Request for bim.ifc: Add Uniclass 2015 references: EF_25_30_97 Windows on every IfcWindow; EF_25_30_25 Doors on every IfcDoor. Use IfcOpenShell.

First a look at what the model holds.

```python
import ifcopenshell

model = ifcopenshell.open("bim.ifc")
print(model.schema)
print("classifications:", [c.Name for c in model.by_type("IfcClassification")])
for ifc_class in ("IfcDoor", "IfcRoof", "IfcStair", "IfcWall", "IfcWindow"):
    print(ifc_class, len(model.by_type(ifc_class)))
```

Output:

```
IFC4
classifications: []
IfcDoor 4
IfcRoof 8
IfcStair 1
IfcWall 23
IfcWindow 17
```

```python
import ifcopenshell
import ifcopenshell.api.classification

model = ifcopenshell.open("bim.ifc")

system = ifcopenshell.api.classification.add_classification(model, classification="Uniclass 2015")

codes = {
    "IfcWindow": ("EF_25_30_97", "Windows"),
    "IfcDoor": ("EF_25_30_25", "Doors"),
}
for ifc_class, (code, name) in codes.items():
    products = model.by_type(ifc_class)
    ifcopenshell.api.classification.add_reference(
        model, products=products, classification=system, identification=code, name=name
    )
    print(code, len(products))

model.write("bim_rev.ifc")
```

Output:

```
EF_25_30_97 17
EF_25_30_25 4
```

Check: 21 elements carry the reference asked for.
